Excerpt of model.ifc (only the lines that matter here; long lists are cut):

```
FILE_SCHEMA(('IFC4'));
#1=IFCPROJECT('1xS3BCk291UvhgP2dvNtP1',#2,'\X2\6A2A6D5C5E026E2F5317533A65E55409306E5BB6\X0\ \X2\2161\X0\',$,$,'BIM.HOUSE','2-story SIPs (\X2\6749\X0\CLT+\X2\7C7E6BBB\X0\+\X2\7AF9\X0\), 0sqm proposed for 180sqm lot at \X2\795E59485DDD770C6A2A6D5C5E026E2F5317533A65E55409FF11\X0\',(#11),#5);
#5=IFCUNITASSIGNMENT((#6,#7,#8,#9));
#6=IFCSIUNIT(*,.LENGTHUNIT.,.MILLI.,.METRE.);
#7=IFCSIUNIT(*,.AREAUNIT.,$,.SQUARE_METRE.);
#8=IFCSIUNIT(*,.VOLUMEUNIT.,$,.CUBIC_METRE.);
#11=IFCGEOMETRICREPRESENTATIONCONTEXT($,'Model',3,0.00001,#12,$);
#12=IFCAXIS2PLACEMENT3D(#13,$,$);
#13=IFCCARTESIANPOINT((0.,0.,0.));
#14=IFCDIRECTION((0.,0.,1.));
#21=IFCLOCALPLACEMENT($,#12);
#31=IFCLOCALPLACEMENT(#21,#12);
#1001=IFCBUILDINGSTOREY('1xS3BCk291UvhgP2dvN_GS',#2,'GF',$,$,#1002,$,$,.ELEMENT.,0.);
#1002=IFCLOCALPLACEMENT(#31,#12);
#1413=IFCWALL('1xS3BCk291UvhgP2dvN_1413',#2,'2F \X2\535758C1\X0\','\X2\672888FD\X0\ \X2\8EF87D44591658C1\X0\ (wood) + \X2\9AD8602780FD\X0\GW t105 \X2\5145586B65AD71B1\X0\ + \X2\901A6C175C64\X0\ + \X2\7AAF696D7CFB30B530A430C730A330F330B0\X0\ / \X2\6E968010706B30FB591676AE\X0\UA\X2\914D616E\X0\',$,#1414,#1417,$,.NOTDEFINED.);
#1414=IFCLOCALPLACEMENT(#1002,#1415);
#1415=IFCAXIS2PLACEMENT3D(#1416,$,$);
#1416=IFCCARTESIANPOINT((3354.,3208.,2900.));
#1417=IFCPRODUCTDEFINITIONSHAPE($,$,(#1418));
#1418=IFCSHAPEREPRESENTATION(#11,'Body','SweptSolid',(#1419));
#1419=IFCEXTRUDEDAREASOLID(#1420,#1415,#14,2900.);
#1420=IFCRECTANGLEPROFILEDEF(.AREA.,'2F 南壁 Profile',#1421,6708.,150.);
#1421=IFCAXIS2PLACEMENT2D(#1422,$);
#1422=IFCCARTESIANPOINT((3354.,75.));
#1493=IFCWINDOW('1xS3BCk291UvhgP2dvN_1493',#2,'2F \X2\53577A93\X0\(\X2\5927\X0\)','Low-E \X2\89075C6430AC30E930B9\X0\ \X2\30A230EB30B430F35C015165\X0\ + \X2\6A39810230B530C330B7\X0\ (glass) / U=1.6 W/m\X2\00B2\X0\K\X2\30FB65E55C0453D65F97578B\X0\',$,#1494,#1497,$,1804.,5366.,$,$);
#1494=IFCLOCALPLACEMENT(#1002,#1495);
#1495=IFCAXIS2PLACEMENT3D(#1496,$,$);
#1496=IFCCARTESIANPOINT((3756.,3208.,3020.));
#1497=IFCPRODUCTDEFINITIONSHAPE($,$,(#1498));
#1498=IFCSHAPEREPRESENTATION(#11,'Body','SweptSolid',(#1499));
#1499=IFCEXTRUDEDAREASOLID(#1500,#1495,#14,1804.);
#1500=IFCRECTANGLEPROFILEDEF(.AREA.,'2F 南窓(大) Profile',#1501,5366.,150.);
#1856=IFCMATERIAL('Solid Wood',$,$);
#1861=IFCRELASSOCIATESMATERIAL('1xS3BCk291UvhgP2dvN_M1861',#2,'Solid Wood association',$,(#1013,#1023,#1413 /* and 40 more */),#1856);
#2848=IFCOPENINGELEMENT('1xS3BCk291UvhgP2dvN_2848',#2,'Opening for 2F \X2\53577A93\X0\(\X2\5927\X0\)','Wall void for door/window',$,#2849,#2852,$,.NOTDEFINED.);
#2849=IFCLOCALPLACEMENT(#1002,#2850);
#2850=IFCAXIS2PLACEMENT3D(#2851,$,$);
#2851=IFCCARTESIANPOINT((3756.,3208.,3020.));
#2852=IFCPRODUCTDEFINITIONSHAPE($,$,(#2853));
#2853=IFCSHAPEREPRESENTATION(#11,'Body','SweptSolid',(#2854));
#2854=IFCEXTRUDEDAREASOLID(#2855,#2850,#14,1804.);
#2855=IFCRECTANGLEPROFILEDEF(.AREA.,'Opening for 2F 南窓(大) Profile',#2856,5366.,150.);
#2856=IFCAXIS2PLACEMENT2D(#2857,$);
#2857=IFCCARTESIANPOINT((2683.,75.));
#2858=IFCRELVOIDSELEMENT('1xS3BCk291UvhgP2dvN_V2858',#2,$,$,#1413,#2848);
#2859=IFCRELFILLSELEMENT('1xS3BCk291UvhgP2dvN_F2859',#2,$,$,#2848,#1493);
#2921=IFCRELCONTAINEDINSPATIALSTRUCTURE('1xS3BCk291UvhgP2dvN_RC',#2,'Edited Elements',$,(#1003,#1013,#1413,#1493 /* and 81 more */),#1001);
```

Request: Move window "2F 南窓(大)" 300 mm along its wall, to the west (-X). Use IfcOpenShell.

```python
import ifcopenshell
import ifcopenshell.api.geometry
import ifcopenshell.util.placement
import ifcopenshell.util.unit

model = ifcopenshell.open("model.ifc")
unit_scale = ifcopenshell.util.unit.calculate_unit_scale(model)

window = model.by_guid("1xS3BCk291UvhgP2dvN_1493")
opening = window.FillsVoids[0].RelatingOpeningElement
wall = opening.VoidsElements[0].RelatingBuildingElement

wall_matrix = ifcopenshell.util.placement.get_local_placement(wall.ObjectPlacement)
shift = wall_matrix[:3, 0] * -0.3 / unit_scale
before = ifcopenshell.util.placement.get_local_placement(window.ObjectPlacement)[:3, 3].copy()

# The window is not placed relative to its opening, so move both.
for product in (opening, window):
    matrix = ifcopenshell.util.placement.get_local_placement(product.ObjectPlacement)
    matrix[:3, 3] += shift
    ifcopenshell.api.geometry.edit_object_placement(model, product=product, matrix=matrix, is_si=False)

after = ifcopenshell.util.placement.get_local_placement(window.ObjectPlacement)[:3, 3]
print("window moved by", (after - before).round(3) + 0.0)

model.write("model-out.ifc")
```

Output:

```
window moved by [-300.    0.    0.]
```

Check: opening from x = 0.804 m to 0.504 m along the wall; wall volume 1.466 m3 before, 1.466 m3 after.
